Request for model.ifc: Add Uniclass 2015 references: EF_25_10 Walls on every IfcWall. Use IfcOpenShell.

First a look at what the model holds.

```python
import ifcopenshell

model = ifcopenshell.open("model.ifc")
print(model.schema)
print("classifications:", [c.Name for c in model.by_type("IfcClassification")])
for ifc_class in ("IfcDoor", "IfcRoof", "IfcStair", "IfcWall", "IfcWindow"):
    print(ifc_class, len(model.by_type(ifc_class)))
```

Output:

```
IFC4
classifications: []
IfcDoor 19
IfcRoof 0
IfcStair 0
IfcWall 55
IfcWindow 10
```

```python
import ifcopenshell
import ifcopenshell.api.classification

model = ifcopenshell.open("model.ifc")

system = ifcopenshell.api.classification.add_classification(model, classification="Uniclass 2015")

codes = {
    "IfcWall": ("EF_25_10", "Walls"),
}
for ifc_class, (code, name) in codes.items():
    products = model.by_type(ifc_class)
    ifcopenshell.api.classification.add_reference(
        model, products=products, classification=system, identification=code, name=name
    )
    print(code, len(products))

model.write("model-out.ifc")
```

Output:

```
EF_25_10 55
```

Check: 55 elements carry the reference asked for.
